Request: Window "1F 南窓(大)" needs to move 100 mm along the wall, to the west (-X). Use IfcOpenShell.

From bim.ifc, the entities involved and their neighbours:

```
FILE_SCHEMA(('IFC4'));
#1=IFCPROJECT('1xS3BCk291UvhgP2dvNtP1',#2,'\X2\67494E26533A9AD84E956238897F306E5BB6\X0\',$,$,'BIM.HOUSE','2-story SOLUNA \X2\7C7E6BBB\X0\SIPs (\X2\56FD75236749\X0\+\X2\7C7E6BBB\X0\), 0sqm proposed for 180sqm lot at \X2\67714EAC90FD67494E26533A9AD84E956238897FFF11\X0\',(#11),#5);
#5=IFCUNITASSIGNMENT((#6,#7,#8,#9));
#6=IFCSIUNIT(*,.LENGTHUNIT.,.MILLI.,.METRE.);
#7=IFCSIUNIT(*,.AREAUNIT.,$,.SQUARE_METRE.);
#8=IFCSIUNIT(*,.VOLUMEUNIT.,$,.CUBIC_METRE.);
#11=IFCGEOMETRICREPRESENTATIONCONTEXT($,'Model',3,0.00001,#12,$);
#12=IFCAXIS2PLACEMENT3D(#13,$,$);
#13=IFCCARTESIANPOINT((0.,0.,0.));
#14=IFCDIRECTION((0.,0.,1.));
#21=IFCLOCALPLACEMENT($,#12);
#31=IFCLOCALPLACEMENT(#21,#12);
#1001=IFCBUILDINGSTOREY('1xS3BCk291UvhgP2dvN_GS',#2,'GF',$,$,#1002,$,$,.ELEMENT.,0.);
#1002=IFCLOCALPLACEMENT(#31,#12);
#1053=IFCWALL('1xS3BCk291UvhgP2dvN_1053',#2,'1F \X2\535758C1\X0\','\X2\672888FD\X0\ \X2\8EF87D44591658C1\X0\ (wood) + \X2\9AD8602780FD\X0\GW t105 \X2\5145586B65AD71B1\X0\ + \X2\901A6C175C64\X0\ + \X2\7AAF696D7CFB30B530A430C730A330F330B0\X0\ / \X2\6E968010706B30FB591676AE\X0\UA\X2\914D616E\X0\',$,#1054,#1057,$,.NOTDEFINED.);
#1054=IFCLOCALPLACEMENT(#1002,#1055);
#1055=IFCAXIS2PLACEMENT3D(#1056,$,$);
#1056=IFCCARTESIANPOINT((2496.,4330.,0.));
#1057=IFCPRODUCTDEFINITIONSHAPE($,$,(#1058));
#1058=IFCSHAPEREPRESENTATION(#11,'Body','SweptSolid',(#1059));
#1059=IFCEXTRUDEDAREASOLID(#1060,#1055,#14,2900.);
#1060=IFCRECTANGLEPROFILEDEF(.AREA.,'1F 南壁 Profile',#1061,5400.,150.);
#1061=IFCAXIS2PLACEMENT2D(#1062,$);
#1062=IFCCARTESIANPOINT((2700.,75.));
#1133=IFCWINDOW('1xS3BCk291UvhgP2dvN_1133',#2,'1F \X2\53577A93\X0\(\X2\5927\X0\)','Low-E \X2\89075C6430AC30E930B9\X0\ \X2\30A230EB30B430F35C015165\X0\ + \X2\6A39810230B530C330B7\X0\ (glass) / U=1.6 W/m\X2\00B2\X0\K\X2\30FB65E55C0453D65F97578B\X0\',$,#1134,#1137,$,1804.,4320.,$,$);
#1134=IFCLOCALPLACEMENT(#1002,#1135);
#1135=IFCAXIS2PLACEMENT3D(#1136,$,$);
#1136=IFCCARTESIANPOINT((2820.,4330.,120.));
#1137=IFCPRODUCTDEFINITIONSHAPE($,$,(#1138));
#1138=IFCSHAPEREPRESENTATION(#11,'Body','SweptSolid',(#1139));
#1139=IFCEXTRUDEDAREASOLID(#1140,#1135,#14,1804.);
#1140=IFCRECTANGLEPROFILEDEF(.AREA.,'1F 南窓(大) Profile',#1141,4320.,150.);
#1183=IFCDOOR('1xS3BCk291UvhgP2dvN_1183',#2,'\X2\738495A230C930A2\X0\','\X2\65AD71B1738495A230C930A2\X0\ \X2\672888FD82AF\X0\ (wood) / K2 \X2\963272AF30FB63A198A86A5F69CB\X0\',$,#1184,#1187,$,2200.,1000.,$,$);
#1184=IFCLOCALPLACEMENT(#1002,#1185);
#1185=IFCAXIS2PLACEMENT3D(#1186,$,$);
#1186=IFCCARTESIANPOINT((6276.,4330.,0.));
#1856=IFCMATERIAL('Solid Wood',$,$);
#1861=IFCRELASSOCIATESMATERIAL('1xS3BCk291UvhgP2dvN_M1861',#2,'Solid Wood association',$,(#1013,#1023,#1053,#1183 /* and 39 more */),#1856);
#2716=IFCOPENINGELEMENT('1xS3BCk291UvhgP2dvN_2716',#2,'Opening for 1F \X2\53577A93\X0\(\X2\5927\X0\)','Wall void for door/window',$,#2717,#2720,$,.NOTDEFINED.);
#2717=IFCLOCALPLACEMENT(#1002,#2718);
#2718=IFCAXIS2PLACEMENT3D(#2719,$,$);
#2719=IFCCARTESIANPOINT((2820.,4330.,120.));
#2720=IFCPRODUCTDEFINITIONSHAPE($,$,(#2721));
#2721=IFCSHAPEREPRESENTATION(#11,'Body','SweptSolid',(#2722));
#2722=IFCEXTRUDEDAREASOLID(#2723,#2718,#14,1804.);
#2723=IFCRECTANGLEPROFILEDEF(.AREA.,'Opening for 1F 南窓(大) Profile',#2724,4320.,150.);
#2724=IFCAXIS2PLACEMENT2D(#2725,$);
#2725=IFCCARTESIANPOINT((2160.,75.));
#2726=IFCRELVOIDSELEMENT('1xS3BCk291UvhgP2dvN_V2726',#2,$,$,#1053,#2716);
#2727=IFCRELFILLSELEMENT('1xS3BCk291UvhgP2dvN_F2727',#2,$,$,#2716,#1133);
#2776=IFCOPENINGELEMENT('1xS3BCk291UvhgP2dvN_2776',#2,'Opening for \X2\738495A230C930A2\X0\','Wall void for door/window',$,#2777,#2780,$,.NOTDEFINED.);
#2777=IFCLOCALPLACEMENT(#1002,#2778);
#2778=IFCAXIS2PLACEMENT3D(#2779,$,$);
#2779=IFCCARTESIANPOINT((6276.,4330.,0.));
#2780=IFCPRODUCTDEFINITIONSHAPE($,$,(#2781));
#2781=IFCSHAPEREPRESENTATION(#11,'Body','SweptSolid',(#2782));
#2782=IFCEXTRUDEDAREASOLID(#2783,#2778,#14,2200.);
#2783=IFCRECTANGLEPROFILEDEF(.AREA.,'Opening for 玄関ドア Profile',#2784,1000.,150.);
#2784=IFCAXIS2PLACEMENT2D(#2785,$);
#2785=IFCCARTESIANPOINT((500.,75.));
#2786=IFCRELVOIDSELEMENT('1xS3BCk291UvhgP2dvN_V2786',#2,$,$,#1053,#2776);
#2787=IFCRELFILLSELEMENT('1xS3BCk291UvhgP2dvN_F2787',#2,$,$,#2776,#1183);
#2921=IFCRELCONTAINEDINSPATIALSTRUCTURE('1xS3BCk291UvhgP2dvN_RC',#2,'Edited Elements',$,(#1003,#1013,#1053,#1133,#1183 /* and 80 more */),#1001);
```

```python
import ifcopenshell
import ifcopenshell.api.geometry
import ifcopenshell.util.placement
import ifcopenshell.util.unit

model = ifcopenshell.open("bim.ifc")
unit_scale = ifcopenshell.util.unit.calculate_unit_scale(model)

window = model.by_id(1133)
opening = window.FillsVoids[0].RelatingOpeningElement
wall = opening.VoidsElements[0].RelatingBuildingElement

wall_matrix = ifcopenshell.util.placement.get_local_placement(wall.ObjectPlacement)
shift = wall_matrix[:3, 0] * -0.1 / unit_scale
before = ifcopenshell.util.placement.get_local_placement(window.ObjectPlacement)[:3, 3].copy()

# The window is not placed relative to its opening, so move both.
for product in (opening, window):
    matrix = ifcopenshell.util.placement.get_local_placement(product.ObjectPlacement)
    matrix[:3, 3] += shift
    ifcopenshell.api.geometry.edit_object_placement(model, product=product, matrix=matrix, is_si=False)

after = ifcopenshell.util.placement.get_local_placement(window.ObjectPlacement)[:3, 3]
print("window moved by", (after - before).round(3) + 0.0)

model.write("bim-out.ifc")
```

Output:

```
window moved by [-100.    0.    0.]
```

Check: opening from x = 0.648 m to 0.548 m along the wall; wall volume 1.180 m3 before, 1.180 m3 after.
